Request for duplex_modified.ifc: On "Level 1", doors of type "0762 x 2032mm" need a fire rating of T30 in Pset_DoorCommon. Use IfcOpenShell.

First a look at what the model holds.

```python
import ifcopenshell
import ifcopenshell.util.element

model = ifcopenshell.open("duplex_modified.ifc")
print(model.schema)
storey = next(s for s in model.by_type("IfcBuildingStorey") if s.Name == "Level 1")
doors = [e for e in ifcopenshell.util.element.get_decomposition(storey) if e.is_a("IfcDoor")]
seen = {}
for e in doors:
    element_type = ifcopenshell.util.element.get_type(e)
    key = (element_type.Name if element_type != e and element_type else None, ifcopenshell.util.element.get_pset(e, "Pset_DoorCommon", "FireRating"))
    seen[key] = seen.get(key, 0) + 1
for (name, value), count in sorted(seen.items(), key=str):
    print(count, "x", name, "|", value)
```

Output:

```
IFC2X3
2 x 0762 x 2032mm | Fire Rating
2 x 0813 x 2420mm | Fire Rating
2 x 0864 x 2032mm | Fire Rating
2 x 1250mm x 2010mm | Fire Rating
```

```python
import ifcopenshell
import ifcopenshell.api.pset
import ifcopenshell.util.element

model = ifcopenshell.open("duplex_modified.ifc")

storey = next(s for s in model.by_type("IfcBuildingStorey") if s.Name == "Level 1")
doors = [e for e in ifcopenshell.util.element.get_decomposition(storey) if e.is_a("IfcDoor")]

count = 0
for e in doors:
    element_type = ifcopenshell.util.element.get_type(e)
    if element_type in (None, e) or element_type.Name != "0762 x 2032mm":
        continue
    # add_pset returns the element's existing set when there is one.
    pset = ifcopenshell.api.pset.add_pset(model, product=e, name="Pset_DoorCommon")
    ifcopenshell.api.pset.edit_pset(model, pset=pset, properties={"FireRating": "T30"})
    count += 1

print(count, "doors updated")

model.write("duplex_modified-out.ifc")
```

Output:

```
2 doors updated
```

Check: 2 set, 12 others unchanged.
